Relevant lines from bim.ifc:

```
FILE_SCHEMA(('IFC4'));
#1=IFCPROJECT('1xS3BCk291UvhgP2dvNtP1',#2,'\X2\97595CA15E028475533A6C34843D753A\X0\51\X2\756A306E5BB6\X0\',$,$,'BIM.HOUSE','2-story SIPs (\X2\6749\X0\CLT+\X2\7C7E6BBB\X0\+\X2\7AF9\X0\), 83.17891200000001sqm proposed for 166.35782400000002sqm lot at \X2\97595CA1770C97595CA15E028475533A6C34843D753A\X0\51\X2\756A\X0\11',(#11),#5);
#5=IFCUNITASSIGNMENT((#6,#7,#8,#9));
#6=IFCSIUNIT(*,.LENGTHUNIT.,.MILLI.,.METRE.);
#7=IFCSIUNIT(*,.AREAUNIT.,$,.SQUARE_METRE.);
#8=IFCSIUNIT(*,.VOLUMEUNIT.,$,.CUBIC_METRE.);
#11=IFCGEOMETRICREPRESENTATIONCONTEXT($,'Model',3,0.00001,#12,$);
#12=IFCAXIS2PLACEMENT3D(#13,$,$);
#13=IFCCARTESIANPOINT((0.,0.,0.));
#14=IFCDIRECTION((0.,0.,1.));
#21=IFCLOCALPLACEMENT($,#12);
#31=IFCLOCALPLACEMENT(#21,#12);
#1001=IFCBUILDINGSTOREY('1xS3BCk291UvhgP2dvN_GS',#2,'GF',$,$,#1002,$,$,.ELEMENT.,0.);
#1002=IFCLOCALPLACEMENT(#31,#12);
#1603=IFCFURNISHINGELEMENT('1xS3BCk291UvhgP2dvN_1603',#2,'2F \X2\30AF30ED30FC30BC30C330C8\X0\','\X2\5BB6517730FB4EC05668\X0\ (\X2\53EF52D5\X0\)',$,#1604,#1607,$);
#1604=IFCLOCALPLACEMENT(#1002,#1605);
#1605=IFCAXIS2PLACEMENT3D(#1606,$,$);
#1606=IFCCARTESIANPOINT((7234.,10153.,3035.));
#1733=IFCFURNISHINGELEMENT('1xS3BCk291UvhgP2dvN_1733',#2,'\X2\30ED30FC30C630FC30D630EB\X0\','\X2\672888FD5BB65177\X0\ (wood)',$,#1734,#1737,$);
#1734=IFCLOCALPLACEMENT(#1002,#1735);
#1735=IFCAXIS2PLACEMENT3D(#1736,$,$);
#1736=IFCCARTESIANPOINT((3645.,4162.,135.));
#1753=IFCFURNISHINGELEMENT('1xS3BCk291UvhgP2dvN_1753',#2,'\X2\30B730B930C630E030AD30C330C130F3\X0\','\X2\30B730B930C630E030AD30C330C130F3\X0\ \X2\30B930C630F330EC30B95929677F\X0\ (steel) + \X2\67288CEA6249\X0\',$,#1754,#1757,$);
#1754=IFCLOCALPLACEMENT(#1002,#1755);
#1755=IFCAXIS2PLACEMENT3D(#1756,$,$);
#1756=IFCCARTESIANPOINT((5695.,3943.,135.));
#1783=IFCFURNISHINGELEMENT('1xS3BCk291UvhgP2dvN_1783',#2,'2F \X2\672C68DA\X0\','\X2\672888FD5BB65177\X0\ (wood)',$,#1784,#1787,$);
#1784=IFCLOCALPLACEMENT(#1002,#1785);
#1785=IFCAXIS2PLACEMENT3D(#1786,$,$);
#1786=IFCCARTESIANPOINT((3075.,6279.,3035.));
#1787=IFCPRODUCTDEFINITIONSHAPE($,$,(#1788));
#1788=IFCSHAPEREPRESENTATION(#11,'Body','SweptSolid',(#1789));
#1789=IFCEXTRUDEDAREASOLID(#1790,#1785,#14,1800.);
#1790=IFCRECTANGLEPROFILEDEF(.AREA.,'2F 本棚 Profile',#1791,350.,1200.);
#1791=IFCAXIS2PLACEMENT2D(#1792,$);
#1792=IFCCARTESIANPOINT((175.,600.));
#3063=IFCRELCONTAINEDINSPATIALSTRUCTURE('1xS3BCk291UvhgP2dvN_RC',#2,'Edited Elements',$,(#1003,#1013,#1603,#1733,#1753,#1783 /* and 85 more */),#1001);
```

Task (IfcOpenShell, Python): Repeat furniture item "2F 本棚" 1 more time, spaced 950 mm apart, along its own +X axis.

```python
import ifcopenshell
import ifcopenshell.api.geometry
import ifcopenshell.api.root
import ifcopenshell.util.element
import ifcopenshell.util.placement

model = ifcopenshell.open("bim.ifc")


def reuse_history(source, copy):
    """copy_class also copies each property set's owner history, people and application; keep the originals."""
    for rel in copy.IsDefinedBy:
        if rel.is_a("IfcRelDefinesByProperties") and (history := rel.RelatingPropertyDefinition.OwnerHistory):
            rel.RelatingPropertyDefinition.OwnerHistory = source.OwnerHistory
            ifcopenshell.util.element.remove_deep2(model, history)


source = model.by_guid("1xS3BCk291UvhgP2dvN_1783")
base = ifcopenshell.util.placement.get_local_placement(source.ObjectPlacement)
step = base[:3, 0] * 950.0

for i in range(1, 2):
    copy = ifcopenshell.api.root.copy_class(model, product=source)
    copy.Representation = ifcopenshell.util.element.copy_deep(
        model, source.Representation, exclude=["IfcGeometricRepresentationContext", "IfcRepresentationMap"]
    )
    reuse_history(source, copy)
    matrix = base.copy()
    matrix[:3, 3] += i * step
    print("added at", matrix[:3, 3].round(3) + 0.0)
    ifcopenshell.api.geometry.edit_object_placement(model, product=copy, matrix=matrix, is_si=False)

model.write("bim_edited.ifc")
```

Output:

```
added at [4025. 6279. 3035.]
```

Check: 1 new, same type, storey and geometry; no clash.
